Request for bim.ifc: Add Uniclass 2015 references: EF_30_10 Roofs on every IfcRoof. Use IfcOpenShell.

First a look at what the model holds.

```python
import ifcopenshell

model = ifcopenshell.open("bim.ifc")
print(model.schema)
print("classifications:", [c.Name for c in model.by_type("IfcClassification")])
for ifc_class in ("IfcDoor", "IfcRoof", "IfcStair", "IfcWall", "IfcWindow"):
    print(ifc_class, len(model.by_type(ifc_class)))
```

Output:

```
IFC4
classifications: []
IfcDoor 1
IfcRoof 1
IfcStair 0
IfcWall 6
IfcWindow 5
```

```python
import ifcopenshell
import ifcopenshell.api.classification

model = ifcopenshell.open("bim.ifc")

system = ifcopenshell.api.classification.add_classification(model, classification="Uniclass 2015")

codes = {
    "IfcRoof": ("EF_30_10", "Roofs"),
}
for ifc_class, (code, name) in codes.items():
    products = model.by_type(ifc_class)
    ifcopenshell.api.classification.add_reference(
        model, products=products, classification=system, identification=code, name=name
    )
    print(code, len(products))

model.write("bim_updated.ifc")
```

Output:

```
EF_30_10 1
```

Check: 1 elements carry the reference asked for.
